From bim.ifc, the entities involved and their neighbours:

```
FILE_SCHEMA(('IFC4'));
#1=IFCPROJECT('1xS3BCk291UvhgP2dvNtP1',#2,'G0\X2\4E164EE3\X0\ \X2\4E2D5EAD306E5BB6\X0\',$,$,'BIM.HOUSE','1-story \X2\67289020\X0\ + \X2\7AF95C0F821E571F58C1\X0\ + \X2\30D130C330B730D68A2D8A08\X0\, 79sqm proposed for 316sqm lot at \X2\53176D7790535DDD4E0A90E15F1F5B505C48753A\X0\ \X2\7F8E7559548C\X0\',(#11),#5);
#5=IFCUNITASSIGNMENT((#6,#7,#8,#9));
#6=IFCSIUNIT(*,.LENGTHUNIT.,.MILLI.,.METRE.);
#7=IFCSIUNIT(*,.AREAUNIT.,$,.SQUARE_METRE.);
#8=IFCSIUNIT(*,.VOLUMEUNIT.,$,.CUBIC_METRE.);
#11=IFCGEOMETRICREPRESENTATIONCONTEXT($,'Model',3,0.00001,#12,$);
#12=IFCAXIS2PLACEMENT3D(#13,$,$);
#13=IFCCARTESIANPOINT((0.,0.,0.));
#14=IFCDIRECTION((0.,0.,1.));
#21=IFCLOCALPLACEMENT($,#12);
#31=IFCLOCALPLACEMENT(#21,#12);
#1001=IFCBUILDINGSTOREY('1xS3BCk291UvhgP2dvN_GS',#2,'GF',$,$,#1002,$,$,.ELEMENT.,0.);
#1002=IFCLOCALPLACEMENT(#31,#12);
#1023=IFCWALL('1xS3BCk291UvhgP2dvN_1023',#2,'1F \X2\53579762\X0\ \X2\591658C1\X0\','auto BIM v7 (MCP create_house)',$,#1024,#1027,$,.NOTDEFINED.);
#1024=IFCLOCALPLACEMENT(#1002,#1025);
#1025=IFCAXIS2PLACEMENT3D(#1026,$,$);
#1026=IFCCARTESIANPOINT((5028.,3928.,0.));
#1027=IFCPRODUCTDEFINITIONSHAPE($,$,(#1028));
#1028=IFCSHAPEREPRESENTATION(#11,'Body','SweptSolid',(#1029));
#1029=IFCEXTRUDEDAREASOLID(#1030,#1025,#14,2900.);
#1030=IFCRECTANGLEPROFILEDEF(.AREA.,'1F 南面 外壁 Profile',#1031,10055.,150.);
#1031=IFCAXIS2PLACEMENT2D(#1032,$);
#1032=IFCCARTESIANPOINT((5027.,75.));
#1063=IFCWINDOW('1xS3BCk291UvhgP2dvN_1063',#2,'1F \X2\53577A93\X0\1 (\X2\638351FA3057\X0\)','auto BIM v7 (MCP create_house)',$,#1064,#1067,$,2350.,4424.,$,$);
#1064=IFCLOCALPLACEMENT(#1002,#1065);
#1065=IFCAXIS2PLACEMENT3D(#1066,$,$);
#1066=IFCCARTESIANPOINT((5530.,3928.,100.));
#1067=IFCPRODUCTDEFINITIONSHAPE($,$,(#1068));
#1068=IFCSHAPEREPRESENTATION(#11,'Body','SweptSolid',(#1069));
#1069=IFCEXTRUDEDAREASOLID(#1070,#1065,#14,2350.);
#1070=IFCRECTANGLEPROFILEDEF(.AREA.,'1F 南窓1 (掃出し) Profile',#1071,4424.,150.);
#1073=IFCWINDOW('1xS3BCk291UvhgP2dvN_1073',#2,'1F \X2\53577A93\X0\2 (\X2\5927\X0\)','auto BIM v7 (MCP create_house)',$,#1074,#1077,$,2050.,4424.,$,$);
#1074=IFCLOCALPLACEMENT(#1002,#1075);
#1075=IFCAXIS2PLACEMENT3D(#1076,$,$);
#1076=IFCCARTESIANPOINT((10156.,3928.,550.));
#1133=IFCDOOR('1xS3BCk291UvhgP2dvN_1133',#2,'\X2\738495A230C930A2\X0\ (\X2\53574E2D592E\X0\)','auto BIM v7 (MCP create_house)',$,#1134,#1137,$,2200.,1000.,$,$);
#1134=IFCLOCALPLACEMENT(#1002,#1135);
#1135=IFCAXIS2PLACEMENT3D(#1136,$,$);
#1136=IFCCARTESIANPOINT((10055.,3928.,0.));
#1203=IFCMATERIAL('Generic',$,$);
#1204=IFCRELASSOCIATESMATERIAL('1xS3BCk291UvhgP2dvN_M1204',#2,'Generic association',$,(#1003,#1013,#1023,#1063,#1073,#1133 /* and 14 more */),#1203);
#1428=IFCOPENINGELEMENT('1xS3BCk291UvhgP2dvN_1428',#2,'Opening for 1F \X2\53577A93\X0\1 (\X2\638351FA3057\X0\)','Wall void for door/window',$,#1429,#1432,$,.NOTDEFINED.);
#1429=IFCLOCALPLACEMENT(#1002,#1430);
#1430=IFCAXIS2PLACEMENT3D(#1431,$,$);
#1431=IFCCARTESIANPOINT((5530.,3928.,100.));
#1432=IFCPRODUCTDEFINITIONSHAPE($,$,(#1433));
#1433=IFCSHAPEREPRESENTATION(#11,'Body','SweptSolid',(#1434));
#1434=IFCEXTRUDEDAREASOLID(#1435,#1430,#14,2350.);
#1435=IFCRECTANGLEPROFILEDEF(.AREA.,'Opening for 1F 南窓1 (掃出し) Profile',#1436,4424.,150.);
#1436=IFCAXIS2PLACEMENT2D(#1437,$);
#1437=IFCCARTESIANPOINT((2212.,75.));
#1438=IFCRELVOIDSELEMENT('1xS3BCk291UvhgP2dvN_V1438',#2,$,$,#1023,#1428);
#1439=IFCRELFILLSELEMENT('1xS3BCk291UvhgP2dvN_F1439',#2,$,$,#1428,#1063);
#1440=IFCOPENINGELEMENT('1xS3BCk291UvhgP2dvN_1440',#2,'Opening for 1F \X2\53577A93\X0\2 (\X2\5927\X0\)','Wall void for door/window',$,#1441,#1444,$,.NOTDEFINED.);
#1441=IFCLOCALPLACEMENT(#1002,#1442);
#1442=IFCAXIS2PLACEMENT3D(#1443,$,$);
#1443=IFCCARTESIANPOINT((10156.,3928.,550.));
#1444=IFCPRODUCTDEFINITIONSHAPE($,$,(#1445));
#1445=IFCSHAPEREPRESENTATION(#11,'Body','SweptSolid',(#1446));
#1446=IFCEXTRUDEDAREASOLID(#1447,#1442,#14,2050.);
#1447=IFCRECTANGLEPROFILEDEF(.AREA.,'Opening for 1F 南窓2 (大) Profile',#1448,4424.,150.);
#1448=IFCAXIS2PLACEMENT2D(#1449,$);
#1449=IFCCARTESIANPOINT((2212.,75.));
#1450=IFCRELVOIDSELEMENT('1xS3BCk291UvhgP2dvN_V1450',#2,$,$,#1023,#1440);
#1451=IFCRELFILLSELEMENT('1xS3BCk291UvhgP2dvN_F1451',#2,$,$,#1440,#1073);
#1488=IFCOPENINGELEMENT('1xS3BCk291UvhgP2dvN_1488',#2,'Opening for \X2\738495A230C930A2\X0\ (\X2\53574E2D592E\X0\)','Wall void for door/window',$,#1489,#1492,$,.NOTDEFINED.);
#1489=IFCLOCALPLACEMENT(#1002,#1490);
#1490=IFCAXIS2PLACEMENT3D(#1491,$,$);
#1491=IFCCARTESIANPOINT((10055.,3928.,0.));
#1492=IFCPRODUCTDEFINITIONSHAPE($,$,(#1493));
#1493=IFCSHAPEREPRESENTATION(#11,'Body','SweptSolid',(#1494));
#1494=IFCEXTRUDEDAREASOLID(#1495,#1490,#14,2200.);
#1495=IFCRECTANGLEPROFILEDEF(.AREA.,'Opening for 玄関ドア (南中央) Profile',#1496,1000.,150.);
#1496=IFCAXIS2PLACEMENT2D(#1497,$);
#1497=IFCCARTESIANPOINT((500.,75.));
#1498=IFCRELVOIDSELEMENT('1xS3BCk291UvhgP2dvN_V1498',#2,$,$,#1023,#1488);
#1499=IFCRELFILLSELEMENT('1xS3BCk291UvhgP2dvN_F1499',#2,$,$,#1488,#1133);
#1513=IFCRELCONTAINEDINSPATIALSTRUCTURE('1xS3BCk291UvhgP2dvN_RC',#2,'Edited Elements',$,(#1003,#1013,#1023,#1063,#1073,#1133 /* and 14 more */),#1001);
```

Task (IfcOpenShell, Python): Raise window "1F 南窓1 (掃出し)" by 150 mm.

```python
import numpy as np
import ifcopenshell
import ifcopenshell.api.geometry
import ifcopenshell.util.placement
import ifcopenshell.util.unit

model = ifcopenshell.open("bim.ifc")
unit_scale = ifcopenshell.util.unit.calculate_unit_scale(model)

window = model.by_id(1063)
opening = window.FillsVoids[0].RelatingOpeningElement
dz = 0.15 / unit_scale

shift = np.array([0.0, 0.0, dz])
# The window is not placed relative to its opening, so move both.
for product in (opening, window):
    matrix = ifcopenshell.util.placement.get_local_placement(product.ObjectPlacement)
    matrix[:3, 3] += shift
    ifcopenshell.api.geometry.edit_object_placement(model, product=product, matrix=matrix, is_si=False)

print(f"moved by {dz * unit_scale:+.3f} m")

model.write("bim_edited.ifc")
```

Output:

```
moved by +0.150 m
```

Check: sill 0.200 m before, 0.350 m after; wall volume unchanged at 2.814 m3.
